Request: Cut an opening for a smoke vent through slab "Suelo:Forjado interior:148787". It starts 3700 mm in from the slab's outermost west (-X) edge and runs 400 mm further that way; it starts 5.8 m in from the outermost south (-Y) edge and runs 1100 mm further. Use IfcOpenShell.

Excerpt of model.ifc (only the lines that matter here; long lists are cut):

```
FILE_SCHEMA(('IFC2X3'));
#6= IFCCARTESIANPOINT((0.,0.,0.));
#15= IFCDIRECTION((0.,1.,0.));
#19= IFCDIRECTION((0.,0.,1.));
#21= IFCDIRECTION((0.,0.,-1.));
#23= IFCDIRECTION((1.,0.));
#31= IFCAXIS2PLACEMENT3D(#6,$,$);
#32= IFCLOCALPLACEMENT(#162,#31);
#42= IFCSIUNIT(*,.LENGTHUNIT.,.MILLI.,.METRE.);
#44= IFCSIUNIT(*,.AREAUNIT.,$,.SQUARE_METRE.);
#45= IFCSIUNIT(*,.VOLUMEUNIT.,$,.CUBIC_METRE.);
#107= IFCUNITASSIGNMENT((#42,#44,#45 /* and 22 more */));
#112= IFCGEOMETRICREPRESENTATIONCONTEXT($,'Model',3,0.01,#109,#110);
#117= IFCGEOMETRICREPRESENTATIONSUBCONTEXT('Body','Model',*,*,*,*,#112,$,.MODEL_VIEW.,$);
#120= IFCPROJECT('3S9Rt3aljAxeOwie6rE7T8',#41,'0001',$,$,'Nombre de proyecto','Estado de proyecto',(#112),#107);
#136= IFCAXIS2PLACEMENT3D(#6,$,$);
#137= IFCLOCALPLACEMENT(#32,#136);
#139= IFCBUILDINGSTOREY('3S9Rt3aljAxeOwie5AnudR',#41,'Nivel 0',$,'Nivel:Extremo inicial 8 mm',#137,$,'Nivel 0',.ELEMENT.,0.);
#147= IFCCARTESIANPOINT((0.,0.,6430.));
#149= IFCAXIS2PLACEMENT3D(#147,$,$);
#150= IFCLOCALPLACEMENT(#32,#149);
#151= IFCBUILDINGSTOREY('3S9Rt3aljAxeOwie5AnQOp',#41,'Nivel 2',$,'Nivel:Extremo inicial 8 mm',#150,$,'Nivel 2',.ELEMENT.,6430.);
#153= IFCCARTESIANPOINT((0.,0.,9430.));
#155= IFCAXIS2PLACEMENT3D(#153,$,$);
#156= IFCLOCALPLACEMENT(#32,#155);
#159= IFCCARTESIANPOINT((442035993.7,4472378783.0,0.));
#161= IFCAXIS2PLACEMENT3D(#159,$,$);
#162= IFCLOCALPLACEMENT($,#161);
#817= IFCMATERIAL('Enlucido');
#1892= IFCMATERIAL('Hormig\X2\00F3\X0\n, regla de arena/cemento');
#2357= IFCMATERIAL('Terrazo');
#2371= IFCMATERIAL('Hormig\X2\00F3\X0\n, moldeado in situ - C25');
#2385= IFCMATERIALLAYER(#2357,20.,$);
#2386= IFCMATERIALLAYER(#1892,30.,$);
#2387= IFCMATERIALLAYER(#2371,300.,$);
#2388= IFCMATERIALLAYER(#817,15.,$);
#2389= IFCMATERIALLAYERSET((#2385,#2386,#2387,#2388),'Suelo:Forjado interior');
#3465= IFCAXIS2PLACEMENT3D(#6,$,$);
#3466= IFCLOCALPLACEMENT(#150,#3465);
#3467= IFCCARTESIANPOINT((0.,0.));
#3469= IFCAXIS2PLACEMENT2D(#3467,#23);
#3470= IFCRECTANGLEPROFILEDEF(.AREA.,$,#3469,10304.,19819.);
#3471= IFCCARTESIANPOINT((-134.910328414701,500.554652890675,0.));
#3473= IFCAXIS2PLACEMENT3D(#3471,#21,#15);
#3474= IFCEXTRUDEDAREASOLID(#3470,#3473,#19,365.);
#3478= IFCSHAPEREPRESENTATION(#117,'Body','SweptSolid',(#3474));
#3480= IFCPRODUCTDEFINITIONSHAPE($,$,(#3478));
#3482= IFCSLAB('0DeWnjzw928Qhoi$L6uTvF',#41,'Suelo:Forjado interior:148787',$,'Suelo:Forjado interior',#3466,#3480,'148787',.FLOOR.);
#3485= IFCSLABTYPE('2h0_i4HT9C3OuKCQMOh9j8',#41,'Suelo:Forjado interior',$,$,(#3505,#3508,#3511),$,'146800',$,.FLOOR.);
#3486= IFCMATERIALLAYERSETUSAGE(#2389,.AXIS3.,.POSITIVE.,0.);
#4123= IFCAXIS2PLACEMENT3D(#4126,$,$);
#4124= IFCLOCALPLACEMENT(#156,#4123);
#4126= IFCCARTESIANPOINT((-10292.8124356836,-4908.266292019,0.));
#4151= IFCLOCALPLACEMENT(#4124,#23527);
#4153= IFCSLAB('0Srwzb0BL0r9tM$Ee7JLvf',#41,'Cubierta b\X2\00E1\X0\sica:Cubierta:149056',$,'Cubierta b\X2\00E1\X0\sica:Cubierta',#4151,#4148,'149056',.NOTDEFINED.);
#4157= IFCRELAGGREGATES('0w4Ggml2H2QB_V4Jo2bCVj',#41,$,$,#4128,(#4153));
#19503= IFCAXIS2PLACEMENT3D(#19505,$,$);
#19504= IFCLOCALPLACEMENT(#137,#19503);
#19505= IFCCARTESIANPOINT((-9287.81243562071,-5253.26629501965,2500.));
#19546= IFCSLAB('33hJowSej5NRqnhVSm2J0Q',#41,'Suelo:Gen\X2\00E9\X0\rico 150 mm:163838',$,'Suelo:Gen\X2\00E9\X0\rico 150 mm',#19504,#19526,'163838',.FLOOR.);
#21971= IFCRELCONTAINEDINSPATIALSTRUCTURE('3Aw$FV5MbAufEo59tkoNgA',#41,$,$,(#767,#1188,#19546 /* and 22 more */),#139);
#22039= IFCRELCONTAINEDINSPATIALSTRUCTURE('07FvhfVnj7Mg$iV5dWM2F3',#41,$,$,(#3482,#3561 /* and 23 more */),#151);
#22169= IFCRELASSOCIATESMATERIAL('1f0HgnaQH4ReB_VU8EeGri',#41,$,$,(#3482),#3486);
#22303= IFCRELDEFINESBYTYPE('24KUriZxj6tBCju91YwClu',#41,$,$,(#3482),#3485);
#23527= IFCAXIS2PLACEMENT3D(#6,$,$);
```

```python
import numpy as np
import ifcopenshell
import ifcopenshell.api.feature
import ifcopenshell.api.geometry
import ifcopenshell.api.root
import ifcopenshell.geom
import ifcopenshell.util.placement
import ifcopenshell.util.representation
import ifcopenshell.util.shape
import ifcopenshell.util.unit

model = ifcopenshell.open("model.ifc")
unit_scale = ifcopenshell.util.unit.calculate_unit_scale(model)
settings = ifcopenshell.geom.settings()


def volume(element):
    """Net volume in cubic metres, openings subtracted."""
    shape = ifcopenshell.geom.create_shape(settings, element)
    return ifcopenshell.util.shape.get_volume(shape.geometry)


slab = model.by_guid("0DeWnjzw928Qhoi$L6uTvF")
before = volume(slab)

# Extent in the slab's own axes, in metres. The edges named are its -X and -Y sides.
slab_shape = ifcopenshell.geom.create_shape(settings, slab)
vertices = ifcopenshell.util.shape.get_vertices(slab_shape.geometry)
x_min, y_min, bottom = vertices.min(axis=0)
top = vertices[:, 2].max()

opening = ifcopenshell.api.root.create_entity(model, ifc_class="IfcOpeningElement", name="Smoke vent opening")
context = ifcopenshell.util.representation.get_context(model, "Model", "Body", "MODEL_VIEW")
width, depth = 0.4, 1.1
outline = [(0.0, 0.0), (width, 0.0), (width, depth), (0.0, depth), (0.0, 0.0)]
# Overshoot both faces by 50 mm so the cut is clean.
shape = ifcopenshell.api.geometry.add_slab_representation(
    model, context=context, depth=top - bottom + 0.1, polyline=outline
)
ifcopenshell.api.geometry.assign_representation(model, product=opening, representation=shape)

matrix = ifcopenshell.util.placement.get_local_placement(slab.ObjectPlacement)
matrix[:, 3] = matrix @ np.append(np.array([x_min + 3.7, y_min + 5.8, bottom - 0.05]) / unit_scale, 1.0)
ifcopenshell.api.geometry.edit_object_placement(model, product=opening, matrix=matrix, is_si=False)
ifcopenshell.api.feature.add_feature(model, feature=opening, element=slab)

after = volume(slab)

print(f"slab volume {before:.3f} -> {after:.3f} m3")

model.write("model_edited.ifc")
```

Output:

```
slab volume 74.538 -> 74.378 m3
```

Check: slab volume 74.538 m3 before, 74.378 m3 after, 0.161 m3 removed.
